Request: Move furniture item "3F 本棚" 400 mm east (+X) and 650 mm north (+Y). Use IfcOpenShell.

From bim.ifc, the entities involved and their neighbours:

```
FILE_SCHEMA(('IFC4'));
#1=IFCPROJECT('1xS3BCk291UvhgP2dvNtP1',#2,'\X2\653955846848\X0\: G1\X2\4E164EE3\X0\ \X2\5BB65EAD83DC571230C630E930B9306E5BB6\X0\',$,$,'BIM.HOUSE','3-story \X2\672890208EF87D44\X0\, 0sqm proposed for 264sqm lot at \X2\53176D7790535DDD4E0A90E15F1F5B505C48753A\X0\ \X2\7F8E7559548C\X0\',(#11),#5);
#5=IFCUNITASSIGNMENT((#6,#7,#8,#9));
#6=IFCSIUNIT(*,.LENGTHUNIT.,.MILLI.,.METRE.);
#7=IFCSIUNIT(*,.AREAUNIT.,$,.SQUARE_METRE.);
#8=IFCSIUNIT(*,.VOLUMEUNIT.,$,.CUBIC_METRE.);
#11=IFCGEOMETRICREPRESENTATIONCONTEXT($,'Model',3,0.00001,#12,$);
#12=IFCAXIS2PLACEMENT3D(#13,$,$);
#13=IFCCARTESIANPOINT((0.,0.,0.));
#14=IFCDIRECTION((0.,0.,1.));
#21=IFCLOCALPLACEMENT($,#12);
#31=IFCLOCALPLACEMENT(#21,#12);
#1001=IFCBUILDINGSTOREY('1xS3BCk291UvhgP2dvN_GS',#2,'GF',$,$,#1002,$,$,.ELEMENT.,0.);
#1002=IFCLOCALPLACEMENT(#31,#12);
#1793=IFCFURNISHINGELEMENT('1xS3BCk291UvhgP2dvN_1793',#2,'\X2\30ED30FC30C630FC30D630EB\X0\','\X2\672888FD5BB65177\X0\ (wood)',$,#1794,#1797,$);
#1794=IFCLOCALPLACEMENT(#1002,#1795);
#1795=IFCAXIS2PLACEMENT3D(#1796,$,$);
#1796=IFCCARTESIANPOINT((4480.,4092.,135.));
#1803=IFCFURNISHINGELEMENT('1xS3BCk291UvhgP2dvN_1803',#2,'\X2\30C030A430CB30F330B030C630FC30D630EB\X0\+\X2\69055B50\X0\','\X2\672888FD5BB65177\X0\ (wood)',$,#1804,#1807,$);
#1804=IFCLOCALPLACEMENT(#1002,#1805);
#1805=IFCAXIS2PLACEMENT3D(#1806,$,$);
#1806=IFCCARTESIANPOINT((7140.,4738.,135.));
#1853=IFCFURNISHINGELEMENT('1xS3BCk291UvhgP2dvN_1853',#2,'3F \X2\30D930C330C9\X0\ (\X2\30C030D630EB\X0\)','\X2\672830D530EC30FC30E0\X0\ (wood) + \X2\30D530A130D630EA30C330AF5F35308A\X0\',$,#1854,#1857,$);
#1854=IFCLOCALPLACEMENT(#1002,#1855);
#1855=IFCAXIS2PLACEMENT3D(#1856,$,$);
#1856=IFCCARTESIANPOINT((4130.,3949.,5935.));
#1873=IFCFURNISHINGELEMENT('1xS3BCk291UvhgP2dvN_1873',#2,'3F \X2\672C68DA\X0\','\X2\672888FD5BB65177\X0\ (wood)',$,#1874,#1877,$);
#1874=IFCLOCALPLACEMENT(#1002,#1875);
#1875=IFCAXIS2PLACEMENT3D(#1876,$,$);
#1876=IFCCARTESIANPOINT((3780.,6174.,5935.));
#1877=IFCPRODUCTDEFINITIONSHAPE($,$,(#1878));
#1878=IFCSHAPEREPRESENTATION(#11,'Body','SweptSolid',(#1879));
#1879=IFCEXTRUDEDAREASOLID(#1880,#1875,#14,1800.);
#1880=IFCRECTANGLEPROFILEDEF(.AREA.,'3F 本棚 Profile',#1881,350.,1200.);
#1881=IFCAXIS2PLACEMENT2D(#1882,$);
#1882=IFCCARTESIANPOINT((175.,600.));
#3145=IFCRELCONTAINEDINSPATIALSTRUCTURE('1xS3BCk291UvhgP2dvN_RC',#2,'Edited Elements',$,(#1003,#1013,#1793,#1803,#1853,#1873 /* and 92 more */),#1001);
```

```python
import ifcopenshell
import ifcopenshell.api.geometry
import ifcopenshell.util.placement
import ifcopenshell.util.unit

model = ifcopenshell.open("bim.ifc")
unit_scale = ifcopenshell.util.unit.calculate_unit_scale(model)

item = model.by_guid("1xS3BCk291UvhgP2dvN_1873")
matrix = ifcopenshell.util.placement.get_local_placement(item.ObjectPlacement)
matrix[0, 3] += 0.4 / unit_scale
matrix[1, 3] += 0.65 / unit_scale
ifcopenshell.api.geometry.edit_object_placement(model, product=item, matrix=matrix, is_si=False)

print(ifcopenshell.util.placement.get_local_placement(item.ObjectPlacement).round(3) + 0.0)

model.write("bim_v2.ifc")
```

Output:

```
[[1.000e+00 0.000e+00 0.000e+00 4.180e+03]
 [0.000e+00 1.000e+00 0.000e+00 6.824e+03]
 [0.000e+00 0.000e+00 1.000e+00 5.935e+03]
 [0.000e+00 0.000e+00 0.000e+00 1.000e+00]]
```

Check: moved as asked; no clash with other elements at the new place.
